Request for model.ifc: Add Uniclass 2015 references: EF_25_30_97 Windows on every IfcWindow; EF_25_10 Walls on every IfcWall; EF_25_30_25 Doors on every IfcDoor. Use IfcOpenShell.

First a look at what the model holds.

```python
import ifcopenshell

model = ifcopenshell.open("model.ifc")
print(model.schema)
print("classifications:", [c.Name for c in model.by_type("IfcClassification")])
for ifc_class in ("IfcDoor", "IfcRoof", "IfcStair", "IfcWall", "IfcWindow"):
    print(ifc_class, len(model.by_type(ifc_class)))
```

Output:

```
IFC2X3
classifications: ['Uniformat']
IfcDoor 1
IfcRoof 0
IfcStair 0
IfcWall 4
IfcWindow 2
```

```python
import ifcopenshell
import ifcopenshell.api.classification

model = ifcopenshell.open("model.ifc")

# IFC2X3 requires Source and Edition and has no link from the project to the system.
system = model.create_entity("IfcClassification", Source="NBS", Edition="2015", Name="Uniclass 2015")

codes = {
    "IfcWindow": ("EF_25_30_97", "Windows"),
    "IfcWall": ("EF_25_10", "Walls"),
    "IfcDoor": ("EF_25_30_25", "Doors"),
}
for ifc_class, (code, name) in codes.items():
    products = model.by_type(ifc_class)
    ifcopenshell.api.classification.add_reference(
        model, products=products, classification=system, identification=code, name=name
    )
    print(code, len(products))

model.write("model_updated.ifc")
```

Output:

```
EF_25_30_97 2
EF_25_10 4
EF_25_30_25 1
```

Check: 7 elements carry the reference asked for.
